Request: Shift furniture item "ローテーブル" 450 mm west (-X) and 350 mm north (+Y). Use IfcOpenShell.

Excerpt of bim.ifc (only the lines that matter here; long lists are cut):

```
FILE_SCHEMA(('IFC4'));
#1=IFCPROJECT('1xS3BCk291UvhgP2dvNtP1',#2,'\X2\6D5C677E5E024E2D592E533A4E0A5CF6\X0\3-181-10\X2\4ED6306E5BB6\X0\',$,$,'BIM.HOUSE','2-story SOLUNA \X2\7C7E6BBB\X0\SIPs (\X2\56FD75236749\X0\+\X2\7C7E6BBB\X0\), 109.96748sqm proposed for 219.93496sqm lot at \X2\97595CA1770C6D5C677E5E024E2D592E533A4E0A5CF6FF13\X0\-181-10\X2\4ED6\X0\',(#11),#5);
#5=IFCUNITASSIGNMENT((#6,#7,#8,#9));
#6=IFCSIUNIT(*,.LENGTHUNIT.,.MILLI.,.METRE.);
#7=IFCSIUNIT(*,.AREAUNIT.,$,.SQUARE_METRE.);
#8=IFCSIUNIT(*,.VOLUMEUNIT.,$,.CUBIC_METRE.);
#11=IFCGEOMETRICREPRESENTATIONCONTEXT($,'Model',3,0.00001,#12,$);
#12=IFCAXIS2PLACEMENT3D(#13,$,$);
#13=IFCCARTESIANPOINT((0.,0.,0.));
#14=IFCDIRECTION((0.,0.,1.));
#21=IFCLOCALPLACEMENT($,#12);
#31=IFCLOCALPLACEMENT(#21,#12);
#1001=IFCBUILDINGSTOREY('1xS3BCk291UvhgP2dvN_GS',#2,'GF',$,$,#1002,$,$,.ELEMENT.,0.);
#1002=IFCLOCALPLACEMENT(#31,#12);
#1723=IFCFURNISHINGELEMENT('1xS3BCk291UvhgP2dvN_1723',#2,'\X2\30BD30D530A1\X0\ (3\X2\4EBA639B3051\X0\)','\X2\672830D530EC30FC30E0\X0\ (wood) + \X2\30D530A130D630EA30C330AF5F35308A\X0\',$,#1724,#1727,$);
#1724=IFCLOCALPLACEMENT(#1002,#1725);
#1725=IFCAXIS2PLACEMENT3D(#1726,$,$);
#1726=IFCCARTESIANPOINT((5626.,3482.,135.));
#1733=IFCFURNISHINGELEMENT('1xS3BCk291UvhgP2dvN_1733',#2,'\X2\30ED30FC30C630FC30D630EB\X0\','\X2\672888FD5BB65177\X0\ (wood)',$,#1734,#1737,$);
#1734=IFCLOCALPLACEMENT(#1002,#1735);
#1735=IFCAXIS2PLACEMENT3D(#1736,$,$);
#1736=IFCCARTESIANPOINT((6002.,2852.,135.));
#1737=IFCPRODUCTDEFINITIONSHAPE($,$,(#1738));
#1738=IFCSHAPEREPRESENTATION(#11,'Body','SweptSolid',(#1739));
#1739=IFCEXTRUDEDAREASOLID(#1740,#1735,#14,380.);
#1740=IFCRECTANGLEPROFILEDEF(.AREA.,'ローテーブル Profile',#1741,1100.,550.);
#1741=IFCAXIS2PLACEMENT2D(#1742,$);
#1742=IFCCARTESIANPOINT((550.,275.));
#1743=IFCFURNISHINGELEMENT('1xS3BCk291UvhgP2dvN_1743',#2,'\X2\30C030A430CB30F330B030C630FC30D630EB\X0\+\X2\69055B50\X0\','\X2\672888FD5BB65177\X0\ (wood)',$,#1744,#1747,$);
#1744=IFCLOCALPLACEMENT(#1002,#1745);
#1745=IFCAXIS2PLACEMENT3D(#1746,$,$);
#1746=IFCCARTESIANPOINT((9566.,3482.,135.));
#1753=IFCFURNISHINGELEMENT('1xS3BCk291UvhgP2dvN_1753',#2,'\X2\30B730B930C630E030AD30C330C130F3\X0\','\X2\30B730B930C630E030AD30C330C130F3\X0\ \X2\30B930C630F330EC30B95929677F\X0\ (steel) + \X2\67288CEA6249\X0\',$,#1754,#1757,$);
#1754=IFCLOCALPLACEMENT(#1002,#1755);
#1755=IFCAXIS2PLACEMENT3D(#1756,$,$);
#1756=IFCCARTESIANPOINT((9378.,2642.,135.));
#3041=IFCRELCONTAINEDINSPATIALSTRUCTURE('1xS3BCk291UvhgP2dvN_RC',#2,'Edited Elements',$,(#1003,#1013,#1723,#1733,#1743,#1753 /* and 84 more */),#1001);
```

```python
import ifcopenshell
import ifcopenshell.api.geometry
import ifcopenshell.util.placement
import ifcopenshell.util.unit

model = ifcopenshell.open("bim.ifc")
unit_scale = ifcopenshell.util.unit.calculate_unit_scale(model)

item = model.by_guid("1xS3BCk291UvhgP2dvN_1733")
matrix = ifcopenshell.util.placement.get_local_placement(item.ObjectPlacement)
matrix[0, 3] -= 0.45 / unit_scale
matrix[1, 3] += 0.35 / unit_scale
ifcopenshell.api.geometry.edit_object_placement(model, product=item, matrix=matrix, is_si=False)

print(ifcopenshell.util.placement.get_local_placement(item.ObjectPlacement).round(3) + 0.0)

model.write("bim_updated.ifc")
```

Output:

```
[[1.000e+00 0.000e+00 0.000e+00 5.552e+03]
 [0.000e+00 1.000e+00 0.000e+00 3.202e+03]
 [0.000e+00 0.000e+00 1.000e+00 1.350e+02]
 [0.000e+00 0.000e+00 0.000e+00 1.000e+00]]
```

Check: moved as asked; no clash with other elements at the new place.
